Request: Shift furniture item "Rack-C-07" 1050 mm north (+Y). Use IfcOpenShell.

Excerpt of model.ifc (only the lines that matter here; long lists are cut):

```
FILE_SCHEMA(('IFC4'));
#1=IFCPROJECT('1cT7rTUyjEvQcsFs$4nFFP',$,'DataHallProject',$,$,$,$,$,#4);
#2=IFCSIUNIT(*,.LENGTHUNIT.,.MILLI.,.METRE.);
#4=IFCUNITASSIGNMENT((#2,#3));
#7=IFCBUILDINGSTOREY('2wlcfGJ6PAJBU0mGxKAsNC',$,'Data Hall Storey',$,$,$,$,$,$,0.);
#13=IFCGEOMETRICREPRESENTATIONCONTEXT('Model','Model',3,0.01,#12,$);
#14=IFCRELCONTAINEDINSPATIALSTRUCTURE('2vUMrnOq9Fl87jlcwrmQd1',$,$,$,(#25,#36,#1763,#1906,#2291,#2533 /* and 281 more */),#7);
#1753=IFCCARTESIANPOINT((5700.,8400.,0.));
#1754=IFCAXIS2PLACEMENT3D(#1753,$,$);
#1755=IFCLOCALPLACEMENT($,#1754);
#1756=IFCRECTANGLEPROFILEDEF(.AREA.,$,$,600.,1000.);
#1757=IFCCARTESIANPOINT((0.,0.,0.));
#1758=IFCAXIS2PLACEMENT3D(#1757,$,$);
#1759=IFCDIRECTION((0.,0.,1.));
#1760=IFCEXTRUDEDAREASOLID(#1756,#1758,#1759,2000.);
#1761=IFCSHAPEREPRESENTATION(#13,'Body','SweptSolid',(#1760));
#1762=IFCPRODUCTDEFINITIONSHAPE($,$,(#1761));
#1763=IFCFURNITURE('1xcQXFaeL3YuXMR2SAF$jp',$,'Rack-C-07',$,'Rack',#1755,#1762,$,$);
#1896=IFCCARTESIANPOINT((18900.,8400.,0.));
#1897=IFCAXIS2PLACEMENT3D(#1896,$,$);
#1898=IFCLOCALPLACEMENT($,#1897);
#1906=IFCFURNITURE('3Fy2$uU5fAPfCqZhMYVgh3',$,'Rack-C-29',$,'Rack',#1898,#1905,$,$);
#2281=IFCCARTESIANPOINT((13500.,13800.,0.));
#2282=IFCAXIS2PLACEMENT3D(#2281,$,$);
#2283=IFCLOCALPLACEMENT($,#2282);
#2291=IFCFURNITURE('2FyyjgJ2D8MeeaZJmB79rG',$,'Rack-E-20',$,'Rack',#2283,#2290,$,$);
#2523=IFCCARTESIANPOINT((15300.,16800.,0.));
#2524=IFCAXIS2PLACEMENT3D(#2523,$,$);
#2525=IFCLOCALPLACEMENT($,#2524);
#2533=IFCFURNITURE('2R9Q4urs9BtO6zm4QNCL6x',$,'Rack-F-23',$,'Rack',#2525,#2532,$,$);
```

```python
import ifcopenshell
import ifcopenshell.api.geometry
import ifcopenshell.util.placement
import ifcopenshell.util.unit

model = ifcopenshell.open("model.ifc")
unit_scale = ifcopenshell.util.unit.calculate_unit_scale(model)

item = model.by_guid("1xcQXFaeL3YuXMR2SAF$jp")
matrix = ifcopenshell.util.placement.get_local_placement(item.ObjectPlacement)
matrix[1, 3] += 1.05 / unit_scale
ifcopenshell.api.geometry.edit_object_placement(model, product=item, matrix=matrix, is_si=False)

print(ifcopenshell.util.placement.get_local_placement(item.ObjectPlacement).round(3) + 0.0)

model.write("model_rev.ifc")
```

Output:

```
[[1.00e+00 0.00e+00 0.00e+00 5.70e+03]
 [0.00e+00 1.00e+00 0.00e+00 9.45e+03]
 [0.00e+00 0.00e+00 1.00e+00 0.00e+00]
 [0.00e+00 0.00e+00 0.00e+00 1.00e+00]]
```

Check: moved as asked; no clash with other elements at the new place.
